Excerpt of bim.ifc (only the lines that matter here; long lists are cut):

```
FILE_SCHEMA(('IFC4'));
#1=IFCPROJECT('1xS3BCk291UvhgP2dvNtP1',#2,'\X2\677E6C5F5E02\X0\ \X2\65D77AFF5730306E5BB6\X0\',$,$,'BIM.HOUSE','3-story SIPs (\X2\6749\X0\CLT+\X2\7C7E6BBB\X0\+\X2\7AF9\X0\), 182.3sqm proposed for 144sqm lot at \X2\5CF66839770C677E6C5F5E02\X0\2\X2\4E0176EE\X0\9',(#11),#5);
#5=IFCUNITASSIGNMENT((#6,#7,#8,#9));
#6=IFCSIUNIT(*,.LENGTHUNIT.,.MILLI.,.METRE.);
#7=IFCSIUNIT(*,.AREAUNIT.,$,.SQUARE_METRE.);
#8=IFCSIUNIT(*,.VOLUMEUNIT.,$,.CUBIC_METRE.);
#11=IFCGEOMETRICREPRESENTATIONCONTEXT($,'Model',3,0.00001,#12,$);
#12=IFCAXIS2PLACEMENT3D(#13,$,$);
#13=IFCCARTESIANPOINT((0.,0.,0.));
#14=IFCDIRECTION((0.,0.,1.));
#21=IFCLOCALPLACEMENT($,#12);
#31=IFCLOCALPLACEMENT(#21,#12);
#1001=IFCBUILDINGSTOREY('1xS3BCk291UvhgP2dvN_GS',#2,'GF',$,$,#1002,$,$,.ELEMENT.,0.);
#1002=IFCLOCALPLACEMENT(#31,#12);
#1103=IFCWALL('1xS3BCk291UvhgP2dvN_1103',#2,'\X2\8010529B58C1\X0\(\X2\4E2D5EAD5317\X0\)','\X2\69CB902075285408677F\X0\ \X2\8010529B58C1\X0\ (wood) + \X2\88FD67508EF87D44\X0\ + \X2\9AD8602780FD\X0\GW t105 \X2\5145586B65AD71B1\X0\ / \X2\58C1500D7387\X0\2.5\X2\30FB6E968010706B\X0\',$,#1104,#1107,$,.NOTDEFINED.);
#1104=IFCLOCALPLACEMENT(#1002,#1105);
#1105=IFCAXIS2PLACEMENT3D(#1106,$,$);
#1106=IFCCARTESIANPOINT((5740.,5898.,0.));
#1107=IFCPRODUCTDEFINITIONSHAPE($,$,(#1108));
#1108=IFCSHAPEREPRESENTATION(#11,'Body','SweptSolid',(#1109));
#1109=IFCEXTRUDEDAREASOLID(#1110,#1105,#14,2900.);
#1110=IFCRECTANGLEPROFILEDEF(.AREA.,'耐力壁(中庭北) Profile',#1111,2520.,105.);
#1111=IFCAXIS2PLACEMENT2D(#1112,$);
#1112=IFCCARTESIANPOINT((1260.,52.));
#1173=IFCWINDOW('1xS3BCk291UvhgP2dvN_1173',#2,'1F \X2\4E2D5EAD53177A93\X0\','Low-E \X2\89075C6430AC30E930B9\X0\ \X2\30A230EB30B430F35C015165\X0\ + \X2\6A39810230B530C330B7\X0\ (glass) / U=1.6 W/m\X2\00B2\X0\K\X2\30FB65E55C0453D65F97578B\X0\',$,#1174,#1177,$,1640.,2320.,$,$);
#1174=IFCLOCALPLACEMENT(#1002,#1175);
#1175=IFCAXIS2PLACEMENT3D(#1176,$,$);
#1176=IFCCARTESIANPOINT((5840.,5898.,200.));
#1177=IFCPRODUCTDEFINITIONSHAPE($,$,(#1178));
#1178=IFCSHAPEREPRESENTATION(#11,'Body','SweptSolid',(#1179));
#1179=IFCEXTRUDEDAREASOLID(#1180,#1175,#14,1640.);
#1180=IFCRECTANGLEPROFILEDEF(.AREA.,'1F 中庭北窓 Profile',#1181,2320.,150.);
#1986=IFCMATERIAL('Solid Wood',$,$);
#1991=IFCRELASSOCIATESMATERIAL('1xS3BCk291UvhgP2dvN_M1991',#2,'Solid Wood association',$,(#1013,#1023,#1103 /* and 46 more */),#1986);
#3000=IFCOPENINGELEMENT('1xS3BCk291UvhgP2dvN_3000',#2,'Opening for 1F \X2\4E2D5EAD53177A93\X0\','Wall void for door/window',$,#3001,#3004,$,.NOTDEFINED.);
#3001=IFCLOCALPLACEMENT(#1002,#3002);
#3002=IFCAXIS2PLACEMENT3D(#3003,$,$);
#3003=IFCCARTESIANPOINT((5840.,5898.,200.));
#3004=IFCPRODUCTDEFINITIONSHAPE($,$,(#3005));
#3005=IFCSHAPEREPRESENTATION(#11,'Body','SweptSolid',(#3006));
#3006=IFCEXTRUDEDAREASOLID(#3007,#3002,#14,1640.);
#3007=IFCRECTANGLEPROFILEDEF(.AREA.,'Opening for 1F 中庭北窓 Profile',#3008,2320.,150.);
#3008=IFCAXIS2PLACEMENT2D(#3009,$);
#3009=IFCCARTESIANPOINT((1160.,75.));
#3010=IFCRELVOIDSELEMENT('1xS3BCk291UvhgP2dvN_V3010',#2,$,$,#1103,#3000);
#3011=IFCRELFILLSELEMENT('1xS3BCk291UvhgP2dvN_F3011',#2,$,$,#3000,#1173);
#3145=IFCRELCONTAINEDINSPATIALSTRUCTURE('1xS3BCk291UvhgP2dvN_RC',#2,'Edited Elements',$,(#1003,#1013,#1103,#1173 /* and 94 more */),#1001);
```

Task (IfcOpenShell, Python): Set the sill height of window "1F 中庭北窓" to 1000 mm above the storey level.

```python
import numpy as np
import ifcopenshell
import ifcopenshell.api.geometry
import ifcopenshell.geom
import ifcopenshell.util.element
import ifcopenshell.util.placement
import ifcopenshell.util.shape
import ifcopenshell.util.unit

model = ifcopenshell.open("bim.ifc")
unit_scale = ifcopenshell.util.unit.calculate_unit_scale(model)

window = model.by_id(1173)
opening = window.FillsVoids[0].RelatingOpeningElement
storey = ifcopenshell.util.element.get_container(window, ifc_class="IfcBuildingStorey")
level = ifcopenshell.util.placement.get_local_placement(storey.ObjectPlacement)[2, 3]

# The opening's origin need not be at the sill, so measure its lowest point.
shape = ifcopenshell.geom.create_shape(ifcopenshell.geom.settings(), opening)
bottom = ifcopenshell.util.shape.get_shape_bottom_elevation(shape, shape.geometry) / unit_scale
dz = level + 1 / unit_scale - bottom

shift = np.array([0.0, 0.0, dz])
# The window is not placed relative to its opening, so move both.
for product in (opening, window):
    matrix = ifcopenshell.util.placement.get_local_placement(product.ObjectPlacement)
    matrix[:3, 3] += shift
    ifcopenshell.api.geometry.edit_object_placement(model, product=product, matrix=matrix, is_si=False)

print(f"moved by {dz * unit_scale:+.3f} m")

model.write("bim_v2.ifc")
```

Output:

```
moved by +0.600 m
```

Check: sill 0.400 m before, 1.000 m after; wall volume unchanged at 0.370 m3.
